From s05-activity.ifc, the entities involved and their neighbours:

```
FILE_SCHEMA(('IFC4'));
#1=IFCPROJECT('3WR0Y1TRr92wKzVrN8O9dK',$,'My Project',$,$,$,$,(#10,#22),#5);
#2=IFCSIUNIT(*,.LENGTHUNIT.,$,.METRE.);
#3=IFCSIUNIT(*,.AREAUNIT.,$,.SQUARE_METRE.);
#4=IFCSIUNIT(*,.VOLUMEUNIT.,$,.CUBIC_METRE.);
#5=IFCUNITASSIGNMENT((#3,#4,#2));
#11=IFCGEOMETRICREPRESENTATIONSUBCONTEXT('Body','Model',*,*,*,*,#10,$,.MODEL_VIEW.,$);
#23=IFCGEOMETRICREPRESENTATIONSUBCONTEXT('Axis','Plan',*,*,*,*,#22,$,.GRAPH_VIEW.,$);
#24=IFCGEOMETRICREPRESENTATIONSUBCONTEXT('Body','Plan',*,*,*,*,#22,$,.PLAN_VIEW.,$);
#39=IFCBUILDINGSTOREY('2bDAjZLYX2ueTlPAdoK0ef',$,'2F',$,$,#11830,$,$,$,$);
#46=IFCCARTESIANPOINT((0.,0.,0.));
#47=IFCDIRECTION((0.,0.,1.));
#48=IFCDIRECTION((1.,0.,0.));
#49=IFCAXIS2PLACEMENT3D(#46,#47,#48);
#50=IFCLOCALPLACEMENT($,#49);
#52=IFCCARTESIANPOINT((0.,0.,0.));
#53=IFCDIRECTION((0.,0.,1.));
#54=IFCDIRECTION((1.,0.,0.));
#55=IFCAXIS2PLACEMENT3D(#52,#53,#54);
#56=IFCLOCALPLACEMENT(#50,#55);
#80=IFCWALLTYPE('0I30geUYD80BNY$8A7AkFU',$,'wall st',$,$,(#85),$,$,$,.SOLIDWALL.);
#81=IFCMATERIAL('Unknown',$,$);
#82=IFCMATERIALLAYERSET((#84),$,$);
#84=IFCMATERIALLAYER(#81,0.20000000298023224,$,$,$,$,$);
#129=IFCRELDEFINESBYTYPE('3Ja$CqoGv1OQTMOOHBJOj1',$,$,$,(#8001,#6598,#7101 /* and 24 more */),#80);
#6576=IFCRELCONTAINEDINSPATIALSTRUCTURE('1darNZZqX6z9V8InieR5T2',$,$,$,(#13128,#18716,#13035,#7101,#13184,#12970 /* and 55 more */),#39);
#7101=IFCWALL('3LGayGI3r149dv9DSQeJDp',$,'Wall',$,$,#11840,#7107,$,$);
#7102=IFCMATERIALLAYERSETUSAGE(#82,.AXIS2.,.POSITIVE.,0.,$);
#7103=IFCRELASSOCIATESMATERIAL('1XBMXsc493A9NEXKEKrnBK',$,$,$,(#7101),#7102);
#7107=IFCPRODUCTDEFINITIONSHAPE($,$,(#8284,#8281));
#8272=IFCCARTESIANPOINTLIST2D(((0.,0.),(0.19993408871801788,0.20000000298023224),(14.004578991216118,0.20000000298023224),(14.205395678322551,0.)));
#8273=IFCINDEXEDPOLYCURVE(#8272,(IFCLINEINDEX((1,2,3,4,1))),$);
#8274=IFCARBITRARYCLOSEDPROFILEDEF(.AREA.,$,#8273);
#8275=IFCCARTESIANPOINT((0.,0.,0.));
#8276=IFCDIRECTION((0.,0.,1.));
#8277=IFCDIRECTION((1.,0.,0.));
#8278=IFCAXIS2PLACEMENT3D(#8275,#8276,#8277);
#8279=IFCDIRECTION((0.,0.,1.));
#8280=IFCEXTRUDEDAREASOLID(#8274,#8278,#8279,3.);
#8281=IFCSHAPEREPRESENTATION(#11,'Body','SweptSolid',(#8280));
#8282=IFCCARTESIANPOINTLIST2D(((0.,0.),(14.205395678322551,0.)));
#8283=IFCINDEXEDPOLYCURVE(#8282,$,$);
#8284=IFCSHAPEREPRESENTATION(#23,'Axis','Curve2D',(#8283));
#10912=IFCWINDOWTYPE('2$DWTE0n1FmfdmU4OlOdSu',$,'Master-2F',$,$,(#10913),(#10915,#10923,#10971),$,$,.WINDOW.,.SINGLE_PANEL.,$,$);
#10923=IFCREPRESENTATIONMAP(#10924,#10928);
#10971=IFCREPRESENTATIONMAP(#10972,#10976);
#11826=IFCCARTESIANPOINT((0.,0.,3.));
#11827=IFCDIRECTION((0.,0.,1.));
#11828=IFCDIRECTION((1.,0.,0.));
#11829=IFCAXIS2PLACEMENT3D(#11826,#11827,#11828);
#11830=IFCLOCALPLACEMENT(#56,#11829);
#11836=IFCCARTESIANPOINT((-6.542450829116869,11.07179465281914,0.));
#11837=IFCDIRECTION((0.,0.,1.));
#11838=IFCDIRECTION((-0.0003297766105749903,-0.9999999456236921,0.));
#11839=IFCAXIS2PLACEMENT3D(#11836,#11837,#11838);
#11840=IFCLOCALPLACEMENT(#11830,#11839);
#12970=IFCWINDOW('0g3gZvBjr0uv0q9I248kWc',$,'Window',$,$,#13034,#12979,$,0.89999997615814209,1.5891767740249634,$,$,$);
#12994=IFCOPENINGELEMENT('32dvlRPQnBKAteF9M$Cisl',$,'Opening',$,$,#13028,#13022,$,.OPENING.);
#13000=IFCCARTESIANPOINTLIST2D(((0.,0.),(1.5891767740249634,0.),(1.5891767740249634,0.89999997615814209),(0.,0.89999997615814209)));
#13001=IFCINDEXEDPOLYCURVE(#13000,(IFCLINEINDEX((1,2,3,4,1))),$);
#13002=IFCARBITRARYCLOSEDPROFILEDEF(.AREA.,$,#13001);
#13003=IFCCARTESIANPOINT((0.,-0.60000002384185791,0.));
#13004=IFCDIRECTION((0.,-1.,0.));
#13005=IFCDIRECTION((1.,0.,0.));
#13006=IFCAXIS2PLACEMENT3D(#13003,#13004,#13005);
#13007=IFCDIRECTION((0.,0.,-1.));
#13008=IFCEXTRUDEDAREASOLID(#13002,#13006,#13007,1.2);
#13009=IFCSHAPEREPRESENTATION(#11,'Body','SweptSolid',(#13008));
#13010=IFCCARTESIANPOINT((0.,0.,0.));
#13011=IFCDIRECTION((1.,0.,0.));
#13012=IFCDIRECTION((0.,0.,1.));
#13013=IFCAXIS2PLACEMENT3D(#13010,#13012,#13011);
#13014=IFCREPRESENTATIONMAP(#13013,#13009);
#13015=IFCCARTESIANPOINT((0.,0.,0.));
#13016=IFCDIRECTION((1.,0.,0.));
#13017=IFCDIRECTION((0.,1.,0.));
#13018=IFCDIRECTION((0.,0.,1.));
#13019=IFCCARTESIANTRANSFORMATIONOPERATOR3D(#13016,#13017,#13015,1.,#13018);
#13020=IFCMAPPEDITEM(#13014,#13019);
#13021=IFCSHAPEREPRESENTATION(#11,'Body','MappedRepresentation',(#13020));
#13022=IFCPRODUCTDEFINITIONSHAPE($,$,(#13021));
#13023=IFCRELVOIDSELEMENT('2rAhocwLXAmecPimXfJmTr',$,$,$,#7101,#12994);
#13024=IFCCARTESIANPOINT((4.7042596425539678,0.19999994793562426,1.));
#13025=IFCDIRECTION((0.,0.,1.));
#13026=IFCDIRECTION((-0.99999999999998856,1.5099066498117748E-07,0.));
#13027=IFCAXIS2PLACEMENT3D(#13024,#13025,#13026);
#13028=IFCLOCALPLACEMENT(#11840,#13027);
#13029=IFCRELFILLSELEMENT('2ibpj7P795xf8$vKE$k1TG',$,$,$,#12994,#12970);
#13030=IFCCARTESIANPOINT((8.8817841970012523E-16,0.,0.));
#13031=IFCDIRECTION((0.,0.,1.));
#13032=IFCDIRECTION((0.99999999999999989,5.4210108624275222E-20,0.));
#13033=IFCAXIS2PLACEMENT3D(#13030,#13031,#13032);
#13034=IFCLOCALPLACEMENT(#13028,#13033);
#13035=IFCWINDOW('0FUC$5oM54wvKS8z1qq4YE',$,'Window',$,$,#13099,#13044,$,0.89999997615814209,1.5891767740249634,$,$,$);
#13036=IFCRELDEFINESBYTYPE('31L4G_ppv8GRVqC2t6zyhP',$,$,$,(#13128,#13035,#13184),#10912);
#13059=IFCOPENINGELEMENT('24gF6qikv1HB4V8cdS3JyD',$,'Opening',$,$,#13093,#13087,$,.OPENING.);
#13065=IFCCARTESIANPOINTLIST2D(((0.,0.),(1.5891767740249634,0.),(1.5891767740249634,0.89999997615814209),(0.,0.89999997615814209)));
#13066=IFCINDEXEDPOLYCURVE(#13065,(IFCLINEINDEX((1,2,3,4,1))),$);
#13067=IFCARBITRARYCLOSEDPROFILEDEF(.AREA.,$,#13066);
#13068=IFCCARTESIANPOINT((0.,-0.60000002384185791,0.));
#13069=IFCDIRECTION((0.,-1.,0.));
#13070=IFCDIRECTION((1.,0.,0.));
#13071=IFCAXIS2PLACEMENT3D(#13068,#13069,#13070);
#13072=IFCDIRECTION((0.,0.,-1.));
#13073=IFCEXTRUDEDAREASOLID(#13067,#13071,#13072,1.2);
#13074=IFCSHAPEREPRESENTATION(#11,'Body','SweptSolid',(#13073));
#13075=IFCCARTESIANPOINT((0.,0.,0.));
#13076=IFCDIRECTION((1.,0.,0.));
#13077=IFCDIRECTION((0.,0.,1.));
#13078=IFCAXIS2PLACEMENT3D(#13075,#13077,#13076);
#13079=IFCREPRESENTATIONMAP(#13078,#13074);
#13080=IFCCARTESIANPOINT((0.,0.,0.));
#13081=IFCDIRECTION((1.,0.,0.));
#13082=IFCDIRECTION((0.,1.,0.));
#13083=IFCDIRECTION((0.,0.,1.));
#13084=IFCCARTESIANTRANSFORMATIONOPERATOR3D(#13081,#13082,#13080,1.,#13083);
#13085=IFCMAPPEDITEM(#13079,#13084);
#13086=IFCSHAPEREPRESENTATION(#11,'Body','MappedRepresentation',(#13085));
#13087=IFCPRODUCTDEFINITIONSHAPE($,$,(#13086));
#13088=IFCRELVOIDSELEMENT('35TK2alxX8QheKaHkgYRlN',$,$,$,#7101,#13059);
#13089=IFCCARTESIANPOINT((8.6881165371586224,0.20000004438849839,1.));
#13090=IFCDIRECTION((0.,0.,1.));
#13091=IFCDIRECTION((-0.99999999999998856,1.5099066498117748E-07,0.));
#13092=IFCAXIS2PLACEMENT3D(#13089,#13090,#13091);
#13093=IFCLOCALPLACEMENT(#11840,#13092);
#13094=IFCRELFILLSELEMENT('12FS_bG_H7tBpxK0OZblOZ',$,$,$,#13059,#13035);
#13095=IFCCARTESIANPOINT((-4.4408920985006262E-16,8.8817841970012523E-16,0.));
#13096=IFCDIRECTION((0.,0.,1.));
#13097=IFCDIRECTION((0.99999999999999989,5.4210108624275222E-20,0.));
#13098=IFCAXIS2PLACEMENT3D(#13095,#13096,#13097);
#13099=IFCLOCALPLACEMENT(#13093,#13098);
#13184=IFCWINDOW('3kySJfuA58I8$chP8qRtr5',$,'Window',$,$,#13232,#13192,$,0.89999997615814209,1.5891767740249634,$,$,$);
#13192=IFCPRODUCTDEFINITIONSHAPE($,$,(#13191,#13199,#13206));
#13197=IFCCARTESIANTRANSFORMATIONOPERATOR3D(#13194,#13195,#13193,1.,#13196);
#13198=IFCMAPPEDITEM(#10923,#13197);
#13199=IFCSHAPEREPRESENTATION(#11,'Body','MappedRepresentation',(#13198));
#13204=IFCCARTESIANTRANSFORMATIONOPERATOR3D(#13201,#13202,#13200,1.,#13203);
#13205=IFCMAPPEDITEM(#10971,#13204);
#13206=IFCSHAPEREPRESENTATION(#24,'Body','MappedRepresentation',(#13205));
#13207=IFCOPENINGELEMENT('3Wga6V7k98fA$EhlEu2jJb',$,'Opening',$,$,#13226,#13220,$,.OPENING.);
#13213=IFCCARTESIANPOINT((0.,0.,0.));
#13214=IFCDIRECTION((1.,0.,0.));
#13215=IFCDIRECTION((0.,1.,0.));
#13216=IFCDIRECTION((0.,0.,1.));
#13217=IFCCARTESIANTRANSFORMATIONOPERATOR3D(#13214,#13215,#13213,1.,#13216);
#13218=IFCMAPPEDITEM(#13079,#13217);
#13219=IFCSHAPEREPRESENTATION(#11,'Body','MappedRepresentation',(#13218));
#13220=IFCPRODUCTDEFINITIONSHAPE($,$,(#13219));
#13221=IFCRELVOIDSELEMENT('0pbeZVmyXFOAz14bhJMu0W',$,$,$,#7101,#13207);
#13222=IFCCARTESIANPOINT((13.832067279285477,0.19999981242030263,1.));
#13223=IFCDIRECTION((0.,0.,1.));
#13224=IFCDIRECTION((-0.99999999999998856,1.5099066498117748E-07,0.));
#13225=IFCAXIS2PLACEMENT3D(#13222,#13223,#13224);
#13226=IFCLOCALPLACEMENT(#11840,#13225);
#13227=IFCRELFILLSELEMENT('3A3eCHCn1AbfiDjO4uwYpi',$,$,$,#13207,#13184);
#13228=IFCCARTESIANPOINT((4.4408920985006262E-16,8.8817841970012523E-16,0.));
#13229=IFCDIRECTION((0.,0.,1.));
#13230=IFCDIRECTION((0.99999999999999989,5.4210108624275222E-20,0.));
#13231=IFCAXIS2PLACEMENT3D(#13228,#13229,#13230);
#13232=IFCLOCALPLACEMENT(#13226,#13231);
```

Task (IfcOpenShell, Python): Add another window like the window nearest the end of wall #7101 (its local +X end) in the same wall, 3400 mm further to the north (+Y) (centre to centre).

```python
import ifcopenshell
import ifcopenshell.api.feature
import ifcopenshell.api.geometry
import ifcopenshell.api.root
import ifcopenshell.geom
import ifcopenshell.util.element
import ifcopenshell.util.placement
import ifcopenshell.util.shape
import ifcopenshell.util.unit

model = ifcopenshell.open("s05-activity.ifc")
unit_scale = ifcopenshell.util.unit.calculate_unit_scale(model)
settings = ifcopenshell.geom.settings()


def volume(element):
    """Net volume in cubic metres, openings subtracted."""
    shape = ifcopenshell.geom.create_shape(settings, element)
    return ifcopenshell.util.shape.get_volume(shape.geometry)


window = model.by_guid("3kySJfuA58I8$chP8qRtr5")
opening = window.FillsVoids[0].RelatingOpeningElement
wall = opening.VoidsElements[0].RelatingBuildingElement
before = volume(wall)
shift = ifcopenshell.util.placement.get_local_placement(wall.ObjectPlacement)[:3, 0] * -3.4 / unit_scale

# copy_class copies the void relationship, type, container and properties, but no geometry.
new_opening = ifcopenshell.api.root.copy_class(model, product=opening)
new_opening.Representation = ifcopenshell.util.element.copy_deep(
    model, opening.Representation, exclude=["IfcGeometricRepresentationContext", "IfcRepresentationMap"]
)
new_window = ifcopenshell.api.root.copy_class(model, product=window)
new_window.Representation = ifcopenshell.util.element.copy_deep(
    model, window.Representation, exclude=["IfcGeometricRepresentationContext", "IfcRepresentationMap"]
)
ifcopenshell.api.feature.add_filling(model, opening=new_opening, element=new_window)

for old, new in ((opening, new_opening), (window, new_window)):
    matrix = ifcopenshell.util.placement.get_local_placement(old.ObjectPlacement)
    matrix[:3, 3] += shift
    ifcopenshell.api.geometry.edit_object_placement(model, product=new, matrix=matrix, is_si=False)

after = volume(wall)

print(f"wall volume {before:.3f} -> {after:.3f} m3")

model.write("s05-activity_rev.ifc")
```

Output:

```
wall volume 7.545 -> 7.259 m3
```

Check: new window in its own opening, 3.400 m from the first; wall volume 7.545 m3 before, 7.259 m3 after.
